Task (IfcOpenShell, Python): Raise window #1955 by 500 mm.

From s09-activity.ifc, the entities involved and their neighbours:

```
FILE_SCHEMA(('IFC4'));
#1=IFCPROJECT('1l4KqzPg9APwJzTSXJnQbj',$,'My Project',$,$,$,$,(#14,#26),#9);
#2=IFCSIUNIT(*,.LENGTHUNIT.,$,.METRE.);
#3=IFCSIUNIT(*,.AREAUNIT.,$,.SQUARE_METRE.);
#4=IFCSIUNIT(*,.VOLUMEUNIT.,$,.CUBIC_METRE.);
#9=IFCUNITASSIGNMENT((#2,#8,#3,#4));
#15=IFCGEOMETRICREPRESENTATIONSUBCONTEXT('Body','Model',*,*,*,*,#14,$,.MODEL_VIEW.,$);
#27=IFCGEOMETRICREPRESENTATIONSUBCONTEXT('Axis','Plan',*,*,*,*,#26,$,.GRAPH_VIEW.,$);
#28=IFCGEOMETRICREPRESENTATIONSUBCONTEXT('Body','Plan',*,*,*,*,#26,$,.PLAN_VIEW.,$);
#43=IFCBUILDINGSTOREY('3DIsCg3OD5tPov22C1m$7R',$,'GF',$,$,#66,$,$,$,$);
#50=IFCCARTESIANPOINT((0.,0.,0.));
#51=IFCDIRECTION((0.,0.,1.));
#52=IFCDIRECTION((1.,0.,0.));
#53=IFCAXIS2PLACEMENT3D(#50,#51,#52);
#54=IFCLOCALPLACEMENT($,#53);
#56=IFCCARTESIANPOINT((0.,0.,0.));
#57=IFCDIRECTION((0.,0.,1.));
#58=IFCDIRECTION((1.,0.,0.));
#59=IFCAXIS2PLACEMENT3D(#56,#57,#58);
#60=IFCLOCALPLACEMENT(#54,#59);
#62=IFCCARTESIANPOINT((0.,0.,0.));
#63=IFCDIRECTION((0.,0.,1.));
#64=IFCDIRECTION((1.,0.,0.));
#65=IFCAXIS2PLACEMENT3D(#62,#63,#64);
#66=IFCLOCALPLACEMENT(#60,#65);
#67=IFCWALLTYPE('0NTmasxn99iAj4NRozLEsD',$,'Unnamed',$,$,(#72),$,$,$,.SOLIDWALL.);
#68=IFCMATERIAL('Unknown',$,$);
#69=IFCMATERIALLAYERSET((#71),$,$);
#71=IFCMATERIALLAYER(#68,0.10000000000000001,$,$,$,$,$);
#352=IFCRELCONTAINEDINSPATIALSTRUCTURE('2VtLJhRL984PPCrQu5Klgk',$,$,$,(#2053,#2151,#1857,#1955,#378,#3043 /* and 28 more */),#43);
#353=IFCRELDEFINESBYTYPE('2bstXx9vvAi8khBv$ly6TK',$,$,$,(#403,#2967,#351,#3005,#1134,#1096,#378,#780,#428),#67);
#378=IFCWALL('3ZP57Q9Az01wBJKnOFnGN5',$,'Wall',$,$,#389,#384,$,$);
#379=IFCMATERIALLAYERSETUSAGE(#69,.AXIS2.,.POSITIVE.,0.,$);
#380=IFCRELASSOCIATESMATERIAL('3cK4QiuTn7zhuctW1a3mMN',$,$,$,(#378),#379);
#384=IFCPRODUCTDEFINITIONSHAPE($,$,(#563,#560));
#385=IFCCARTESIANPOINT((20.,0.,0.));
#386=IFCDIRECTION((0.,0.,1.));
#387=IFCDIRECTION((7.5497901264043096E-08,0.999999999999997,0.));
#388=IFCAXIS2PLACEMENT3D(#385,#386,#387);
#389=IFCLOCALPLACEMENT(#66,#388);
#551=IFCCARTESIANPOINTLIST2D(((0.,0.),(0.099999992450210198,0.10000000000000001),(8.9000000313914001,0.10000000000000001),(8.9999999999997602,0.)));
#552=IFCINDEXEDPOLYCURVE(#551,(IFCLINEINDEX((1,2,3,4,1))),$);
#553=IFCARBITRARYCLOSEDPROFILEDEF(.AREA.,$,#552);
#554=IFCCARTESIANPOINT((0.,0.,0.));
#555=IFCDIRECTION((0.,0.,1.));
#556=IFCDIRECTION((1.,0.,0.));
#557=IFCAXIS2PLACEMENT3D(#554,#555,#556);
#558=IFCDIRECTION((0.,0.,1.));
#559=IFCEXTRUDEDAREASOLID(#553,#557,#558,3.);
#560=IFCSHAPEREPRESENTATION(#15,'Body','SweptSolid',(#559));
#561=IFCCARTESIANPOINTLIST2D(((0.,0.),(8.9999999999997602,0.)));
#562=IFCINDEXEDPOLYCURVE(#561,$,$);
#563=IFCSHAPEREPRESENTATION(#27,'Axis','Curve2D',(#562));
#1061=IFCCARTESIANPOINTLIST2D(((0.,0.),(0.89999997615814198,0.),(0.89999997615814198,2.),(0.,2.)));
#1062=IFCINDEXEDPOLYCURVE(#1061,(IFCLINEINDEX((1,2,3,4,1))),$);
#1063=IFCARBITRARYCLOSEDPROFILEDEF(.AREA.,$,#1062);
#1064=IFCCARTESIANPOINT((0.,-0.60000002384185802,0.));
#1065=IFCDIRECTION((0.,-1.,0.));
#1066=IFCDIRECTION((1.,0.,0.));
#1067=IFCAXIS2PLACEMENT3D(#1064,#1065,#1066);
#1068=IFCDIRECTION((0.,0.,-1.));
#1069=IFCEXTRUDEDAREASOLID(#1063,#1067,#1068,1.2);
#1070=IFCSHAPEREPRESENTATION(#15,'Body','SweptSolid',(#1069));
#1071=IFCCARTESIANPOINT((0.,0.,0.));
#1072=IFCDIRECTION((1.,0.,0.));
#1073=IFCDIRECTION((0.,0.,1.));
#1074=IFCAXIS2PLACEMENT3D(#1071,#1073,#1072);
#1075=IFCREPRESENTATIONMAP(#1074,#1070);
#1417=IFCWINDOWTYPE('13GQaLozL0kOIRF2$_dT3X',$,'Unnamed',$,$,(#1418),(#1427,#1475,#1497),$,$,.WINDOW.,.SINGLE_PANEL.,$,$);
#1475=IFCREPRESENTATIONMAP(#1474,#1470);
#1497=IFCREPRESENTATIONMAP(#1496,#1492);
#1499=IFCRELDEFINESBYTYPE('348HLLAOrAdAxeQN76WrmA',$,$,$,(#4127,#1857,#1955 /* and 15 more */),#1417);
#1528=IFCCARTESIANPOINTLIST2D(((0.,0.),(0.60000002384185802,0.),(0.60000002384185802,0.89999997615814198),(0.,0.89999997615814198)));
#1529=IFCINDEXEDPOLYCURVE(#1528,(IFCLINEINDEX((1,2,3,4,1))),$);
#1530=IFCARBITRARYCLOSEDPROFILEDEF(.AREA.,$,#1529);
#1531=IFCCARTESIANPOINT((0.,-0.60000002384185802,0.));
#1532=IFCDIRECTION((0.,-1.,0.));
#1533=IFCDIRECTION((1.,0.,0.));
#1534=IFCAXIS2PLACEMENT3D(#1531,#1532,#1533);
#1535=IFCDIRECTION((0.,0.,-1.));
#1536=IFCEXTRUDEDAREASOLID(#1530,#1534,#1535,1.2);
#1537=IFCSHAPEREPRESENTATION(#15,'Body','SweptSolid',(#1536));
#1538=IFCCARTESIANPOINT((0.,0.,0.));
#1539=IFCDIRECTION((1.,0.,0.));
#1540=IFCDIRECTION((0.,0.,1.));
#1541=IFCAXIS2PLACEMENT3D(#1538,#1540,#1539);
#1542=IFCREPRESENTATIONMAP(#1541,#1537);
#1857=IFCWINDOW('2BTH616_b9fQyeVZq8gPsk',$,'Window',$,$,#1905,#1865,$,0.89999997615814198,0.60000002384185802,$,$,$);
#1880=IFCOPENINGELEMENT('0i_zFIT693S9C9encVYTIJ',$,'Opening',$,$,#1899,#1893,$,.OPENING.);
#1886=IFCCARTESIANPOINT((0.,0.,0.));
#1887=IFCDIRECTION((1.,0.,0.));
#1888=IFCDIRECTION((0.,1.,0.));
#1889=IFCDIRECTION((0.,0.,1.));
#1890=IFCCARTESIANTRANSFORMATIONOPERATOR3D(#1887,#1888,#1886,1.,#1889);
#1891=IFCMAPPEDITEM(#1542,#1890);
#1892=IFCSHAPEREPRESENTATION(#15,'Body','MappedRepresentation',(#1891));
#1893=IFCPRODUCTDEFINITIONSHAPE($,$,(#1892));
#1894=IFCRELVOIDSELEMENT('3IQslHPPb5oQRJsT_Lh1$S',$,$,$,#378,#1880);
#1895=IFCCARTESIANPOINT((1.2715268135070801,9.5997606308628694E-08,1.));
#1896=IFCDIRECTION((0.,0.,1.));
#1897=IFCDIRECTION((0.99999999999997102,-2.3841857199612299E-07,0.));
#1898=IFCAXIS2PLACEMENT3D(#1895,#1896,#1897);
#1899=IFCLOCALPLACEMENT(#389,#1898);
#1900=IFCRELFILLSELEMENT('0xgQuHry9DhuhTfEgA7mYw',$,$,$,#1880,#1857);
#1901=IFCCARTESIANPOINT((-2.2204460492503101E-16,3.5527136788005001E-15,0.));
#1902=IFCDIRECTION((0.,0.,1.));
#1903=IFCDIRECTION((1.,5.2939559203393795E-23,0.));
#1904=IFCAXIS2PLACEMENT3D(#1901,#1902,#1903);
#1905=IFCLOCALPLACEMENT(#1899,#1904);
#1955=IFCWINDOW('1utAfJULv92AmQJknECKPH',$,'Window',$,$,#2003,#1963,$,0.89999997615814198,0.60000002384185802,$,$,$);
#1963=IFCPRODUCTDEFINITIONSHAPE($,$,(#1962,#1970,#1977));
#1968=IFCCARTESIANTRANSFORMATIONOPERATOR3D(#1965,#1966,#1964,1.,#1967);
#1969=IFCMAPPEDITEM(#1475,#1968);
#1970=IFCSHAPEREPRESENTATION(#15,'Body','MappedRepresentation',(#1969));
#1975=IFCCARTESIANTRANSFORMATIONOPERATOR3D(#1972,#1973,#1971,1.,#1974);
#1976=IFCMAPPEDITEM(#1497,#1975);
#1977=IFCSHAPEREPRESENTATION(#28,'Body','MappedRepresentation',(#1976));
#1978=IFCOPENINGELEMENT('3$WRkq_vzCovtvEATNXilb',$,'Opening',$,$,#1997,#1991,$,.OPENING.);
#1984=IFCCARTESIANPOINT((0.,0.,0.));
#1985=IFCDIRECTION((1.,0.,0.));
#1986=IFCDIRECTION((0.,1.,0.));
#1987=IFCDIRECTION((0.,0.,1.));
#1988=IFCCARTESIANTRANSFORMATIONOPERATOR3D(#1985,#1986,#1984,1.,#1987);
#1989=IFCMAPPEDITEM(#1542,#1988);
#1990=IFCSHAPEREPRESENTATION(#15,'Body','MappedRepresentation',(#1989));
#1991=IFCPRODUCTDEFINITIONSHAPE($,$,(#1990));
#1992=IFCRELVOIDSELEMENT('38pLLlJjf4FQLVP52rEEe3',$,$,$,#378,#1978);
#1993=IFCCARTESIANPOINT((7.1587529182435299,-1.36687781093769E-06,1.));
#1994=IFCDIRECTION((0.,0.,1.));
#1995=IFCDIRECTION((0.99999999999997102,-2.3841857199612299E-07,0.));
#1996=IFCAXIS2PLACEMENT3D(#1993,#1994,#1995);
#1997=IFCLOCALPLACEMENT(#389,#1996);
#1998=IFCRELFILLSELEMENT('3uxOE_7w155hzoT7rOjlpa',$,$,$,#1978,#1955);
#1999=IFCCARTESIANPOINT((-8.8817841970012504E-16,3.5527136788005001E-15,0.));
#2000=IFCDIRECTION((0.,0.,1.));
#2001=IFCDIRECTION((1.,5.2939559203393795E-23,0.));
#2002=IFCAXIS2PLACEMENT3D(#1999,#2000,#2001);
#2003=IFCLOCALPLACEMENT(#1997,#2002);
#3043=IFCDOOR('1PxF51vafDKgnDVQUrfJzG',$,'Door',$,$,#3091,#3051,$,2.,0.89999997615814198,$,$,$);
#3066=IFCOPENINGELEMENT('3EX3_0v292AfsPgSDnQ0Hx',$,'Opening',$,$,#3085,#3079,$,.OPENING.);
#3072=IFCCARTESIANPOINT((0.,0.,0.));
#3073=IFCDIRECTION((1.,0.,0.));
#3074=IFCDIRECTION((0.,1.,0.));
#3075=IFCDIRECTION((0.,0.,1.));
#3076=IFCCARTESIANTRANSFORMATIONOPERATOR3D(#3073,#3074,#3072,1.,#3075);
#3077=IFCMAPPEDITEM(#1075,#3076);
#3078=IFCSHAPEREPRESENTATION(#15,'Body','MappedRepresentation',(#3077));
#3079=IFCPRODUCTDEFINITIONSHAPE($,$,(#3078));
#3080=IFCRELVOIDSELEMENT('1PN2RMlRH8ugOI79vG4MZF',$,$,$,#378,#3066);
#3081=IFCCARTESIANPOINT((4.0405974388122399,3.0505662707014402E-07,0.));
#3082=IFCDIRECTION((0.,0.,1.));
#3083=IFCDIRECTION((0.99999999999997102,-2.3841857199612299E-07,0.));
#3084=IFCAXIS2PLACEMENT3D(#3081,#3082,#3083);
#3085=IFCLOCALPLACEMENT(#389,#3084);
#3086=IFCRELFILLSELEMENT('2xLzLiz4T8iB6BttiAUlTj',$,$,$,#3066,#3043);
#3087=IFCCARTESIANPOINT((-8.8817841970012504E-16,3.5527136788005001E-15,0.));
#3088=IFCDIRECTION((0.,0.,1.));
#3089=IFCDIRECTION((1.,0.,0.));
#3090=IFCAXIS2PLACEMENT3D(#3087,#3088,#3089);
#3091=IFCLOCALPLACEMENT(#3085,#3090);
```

```python
import numpy as np
import ifcopenshell
import ifcopenshell.api.geometry
import ifcopenshell.util.placement
import ifcopenshell.util.unit

model = ifcopenshell.open("s09-activity.ifc")
unit_scale = ifcopenshell.util.unit.calculate_unit_scale(model)

window = model.by_guid("1utAfJULv92AmQJknECKPH")
opening = window.FillsVoids[0].RelatingOpeningElement
dz = 0.5 / unit_scale

shift = np.array([0.0, 0.0, dz])
# The window is placed relative to its opening, so it follows when the opening moves.
matrix = ifcopenshell.util.placement.get_local_placement(opening.ObjectPlacement)
matrix[:3, 3] += shift
ifcopenshell.api.geometry.edit_object_placement(
    model, product=opening, matrix=matrix, is_si=False, should_transform_children=True
)

print(f"moved by {dz * unit_scale:+.3f} m")

model.write("s09-activity_rev.ifc")
```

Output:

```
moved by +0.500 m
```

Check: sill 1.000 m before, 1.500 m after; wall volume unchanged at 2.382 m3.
